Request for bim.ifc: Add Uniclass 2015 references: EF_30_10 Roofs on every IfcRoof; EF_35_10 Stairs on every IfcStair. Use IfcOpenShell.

First a look at what the model holds.

```python
import ifcopenshell

model = ifcopenshell.open("bim.ifc")
print(model.schema)
print("classifications:", [c.Name for c in model.by_type("IfcClassification")])
for ifc_class in ("IfcDoor", "IfcRoof", "IfcStair", "IfcWall", "IfcWindow"):
    print(ifc_class, len(model.by_type(ifc_class)))
```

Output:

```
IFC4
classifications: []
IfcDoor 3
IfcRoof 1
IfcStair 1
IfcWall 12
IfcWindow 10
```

```python
import ifcopenshell
import ifcopenshell.api.classification

model = ifcopenshell.open("bim.ifc")

system = ifcopenshell.api.classification.add_classification(model, classification="Uniclass 2015")

codes = {
    "IfcRoof": ("EF_30_10", "Roofs"),
    "IfcStair": ("EF_35_10", "Stairs"),
}
for ifc_class, (code, name) in codes.items():
    products = model.by_type(ifc_class)
    ifcopenshell.api.classification.add_reference(
        model, products=products, classification=system, identification=code, name=name
    )
    print(code, len(products))

model.write("bim_edited.ifc")
```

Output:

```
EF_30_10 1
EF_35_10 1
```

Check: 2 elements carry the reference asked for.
